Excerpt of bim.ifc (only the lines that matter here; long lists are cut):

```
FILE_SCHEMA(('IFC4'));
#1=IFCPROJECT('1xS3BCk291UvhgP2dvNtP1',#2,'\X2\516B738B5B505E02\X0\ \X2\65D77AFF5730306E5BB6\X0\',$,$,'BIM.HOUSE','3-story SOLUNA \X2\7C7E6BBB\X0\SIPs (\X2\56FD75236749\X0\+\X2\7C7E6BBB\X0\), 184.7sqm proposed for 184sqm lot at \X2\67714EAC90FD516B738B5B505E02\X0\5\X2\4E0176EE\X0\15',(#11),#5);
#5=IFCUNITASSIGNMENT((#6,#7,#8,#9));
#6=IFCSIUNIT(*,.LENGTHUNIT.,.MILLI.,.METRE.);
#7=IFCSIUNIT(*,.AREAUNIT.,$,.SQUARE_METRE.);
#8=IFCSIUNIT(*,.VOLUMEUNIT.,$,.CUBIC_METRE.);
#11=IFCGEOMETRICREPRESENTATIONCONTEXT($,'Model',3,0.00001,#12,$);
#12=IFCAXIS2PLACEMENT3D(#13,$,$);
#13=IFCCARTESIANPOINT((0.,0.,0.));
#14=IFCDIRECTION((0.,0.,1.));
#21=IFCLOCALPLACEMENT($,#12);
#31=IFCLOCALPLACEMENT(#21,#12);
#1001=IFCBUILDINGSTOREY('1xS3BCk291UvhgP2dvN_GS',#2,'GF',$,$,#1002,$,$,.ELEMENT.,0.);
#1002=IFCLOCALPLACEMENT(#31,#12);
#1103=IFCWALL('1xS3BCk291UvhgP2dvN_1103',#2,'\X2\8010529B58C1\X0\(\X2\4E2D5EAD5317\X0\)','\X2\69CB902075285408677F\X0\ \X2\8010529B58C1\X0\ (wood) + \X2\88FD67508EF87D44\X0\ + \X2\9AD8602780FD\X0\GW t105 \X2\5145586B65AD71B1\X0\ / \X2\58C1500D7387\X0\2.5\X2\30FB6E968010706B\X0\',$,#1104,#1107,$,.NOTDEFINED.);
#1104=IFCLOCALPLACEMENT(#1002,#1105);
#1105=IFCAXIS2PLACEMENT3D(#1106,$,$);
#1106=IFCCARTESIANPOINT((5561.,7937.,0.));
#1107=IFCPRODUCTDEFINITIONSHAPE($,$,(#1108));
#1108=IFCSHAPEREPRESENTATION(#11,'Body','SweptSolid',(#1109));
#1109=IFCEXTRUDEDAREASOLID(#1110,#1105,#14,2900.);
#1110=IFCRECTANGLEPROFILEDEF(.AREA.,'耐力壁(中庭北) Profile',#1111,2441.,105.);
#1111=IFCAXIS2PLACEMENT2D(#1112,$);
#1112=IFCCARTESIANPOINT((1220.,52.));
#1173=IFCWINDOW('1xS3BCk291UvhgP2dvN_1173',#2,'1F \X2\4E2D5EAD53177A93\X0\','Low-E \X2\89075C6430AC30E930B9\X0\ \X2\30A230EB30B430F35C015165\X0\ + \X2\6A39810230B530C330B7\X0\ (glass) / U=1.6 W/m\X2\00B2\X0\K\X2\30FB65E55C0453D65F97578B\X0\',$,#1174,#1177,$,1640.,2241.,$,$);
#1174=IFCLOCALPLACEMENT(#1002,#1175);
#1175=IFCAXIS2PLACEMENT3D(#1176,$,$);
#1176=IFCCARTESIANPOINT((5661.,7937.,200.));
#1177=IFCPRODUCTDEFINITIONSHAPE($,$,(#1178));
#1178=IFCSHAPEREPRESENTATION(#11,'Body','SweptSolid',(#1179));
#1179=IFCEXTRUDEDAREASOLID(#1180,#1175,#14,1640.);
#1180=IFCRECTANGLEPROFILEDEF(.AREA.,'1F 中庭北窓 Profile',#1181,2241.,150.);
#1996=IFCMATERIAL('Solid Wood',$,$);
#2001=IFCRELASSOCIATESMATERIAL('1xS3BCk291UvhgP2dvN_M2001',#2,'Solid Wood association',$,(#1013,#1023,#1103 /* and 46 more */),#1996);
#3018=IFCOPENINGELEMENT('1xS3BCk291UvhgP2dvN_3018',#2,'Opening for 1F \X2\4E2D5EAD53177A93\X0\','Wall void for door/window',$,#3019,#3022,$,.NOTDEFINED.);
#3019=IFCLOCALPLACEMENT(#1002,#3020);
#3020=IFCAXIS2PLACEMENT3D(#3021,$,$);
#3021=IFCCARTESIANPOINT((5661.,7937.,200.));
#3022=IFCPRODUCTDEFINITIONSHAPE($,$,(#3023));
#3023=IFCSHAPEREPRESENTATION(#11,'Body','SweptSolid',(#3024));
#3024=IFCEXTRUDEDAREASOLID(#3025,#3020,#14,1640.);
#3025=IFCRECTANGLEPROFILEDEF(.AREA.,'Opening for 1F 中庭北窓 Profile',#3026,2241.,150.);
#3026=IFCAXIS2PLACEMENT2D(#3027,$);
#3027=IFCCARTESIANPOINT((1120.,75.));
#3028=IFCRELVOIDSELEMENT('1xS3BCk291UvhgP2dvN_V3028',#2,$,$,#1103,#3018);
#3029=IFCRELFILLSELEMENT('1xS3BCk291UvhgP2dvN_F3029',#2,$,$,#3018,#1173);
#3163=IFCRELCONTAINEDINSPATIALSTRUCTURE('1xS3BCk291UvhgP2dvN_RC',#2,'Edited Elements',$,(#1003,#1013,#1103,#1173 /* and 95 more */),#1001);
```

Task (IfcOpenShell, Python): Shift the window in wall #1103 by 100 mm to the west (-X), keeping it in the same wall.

```python
import ifcopenshell
import ifcopenshell.api.geometry
import ifcopenshell.util.placement
import ifcopenshell.util.unit

model = ifcopenshell.open("bim.ifc")
unit_scale = ifcopenshell.util.unit.calculate_unit_scale(model)

window = model.by_guid("1xS3BCk291UvhgP2dvN_1173")
opening = window.FillsVoids[0].RelatingOpeningElement
wall = opening.VoidsElements[0].RelatingBuildingElement

wall_matrix = ifcopenshell.util.placement.get_local_placement(wall.ObjectPlacement)
shift = wall_matrix[:3, 0] * -0.1 / unit_scale
before = ifcopenshell.util.placement.get_local_placement(window.ObjectPlacement)[:3, 3].copy()

# The window is not placed relative to its opening, so move both.
for product in (opening, window):
    matrix = ifcopenshell.util.placement.get_local_placement(product.ObjectPlacement)
    matrix[:3, 3] += shift
    ifcopenshell.api.geometry.edit_object_placement(model, product=product, matrix=matrix, is_si=False)

after = ifcopenshell.util.placement.get_local_placement(window.ObjectPlacement)[:3, 3]
print("window moved by", (after - before).round(3) + 0.0)

model.write("bim_rev.ifc")
```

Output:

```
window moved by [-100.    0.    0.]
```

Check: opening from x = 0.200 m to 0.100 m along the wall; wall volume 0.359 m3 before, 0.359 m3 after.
